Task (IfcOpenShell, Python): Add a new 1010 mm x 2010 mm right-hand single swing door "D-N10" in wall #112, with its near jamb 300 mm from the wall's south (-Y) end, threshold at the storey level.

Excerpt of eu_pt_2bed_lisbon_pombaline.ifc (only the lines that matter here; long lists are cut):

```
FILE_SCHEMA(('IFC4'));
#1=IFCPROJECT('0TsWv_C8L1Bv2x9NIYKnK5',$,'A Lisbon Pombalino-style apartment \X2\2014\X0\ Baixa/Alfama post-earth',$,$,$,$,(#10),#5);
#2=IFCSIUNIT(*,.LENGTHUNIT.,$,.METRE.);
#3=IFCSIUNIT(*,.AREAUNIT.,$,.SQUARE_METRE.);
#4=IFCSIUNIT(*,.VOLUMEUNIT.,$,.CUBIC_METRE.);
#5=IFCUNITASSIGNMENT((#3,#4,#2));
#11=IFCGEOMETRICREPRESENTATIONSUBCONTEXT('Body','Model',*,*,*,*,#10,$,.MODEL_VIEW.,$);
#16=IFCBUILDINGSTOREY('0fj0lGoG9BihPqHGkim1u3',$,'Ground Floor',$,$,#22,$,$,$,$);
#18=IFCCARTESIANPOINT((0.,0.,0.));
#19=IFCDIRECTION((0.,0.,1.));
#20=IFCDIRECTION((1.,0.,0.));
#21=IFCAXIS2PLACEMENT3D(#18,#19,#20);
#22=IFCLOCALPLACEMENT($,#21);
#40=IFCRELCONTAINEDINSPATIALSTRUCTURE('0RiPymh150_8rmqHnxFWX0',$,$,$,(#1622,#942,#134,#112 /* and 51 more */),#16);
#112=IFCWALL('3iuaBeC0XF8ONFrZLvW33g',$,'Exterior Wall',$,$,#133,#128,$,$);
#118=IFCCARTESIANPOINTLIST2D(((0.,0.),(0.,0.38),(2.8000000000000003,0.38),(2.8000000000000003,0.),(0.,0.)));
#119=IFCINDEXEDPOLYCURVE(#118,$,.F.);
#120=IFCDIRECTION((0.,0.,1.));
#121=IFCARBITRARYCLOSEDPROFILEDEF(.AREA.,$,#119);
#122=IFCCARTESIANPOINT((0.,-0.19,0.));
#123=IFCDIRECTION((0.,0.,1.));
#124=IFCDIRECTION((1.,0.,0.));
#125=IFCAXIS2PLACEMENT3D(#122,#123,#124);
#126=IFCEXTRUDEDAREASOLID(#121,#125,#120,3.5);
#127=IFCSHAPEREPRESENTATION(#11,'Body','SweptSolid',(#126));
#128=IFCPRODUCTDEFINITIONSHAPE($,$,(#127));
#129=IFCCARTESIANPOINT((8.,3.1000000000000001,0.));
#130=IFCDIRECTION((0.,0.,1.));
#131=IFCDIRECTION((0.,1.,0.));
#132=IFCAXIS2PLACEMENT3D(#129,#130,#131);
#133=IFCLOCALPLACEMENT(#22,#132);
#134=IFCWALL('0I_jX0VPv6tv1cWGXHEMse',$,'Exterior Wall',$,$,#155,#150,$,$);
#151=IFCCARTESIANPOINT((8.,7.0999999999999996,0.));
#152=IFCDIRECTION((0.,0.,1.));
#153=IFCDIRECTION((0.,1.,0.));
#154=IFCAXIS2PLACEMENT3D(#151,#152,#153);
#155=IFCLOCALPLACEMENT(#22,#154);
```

```python
import numpy as np
import ifcopenshell
import ifcopenshell.api.feature
import ifcopenshell.api.geometry
import ifcopenshell.api.root
import ifcopenshell.api.spatial
import ifcopenshell.geom
import ifcopenshell.util.element
import ifcopenshell.util.placement
import ifcopenshell.util.representation
import ifcopenshell.util.shape
import ifcopenshell.util.unit

model = ifcopenshell.open("eu_pt_2bed_lisbon_pombaline.ifc")
unit_scale = ifcopenshell.util.unit.calculate_unit_scale(model)
settings = ifcopenshell.geom.settings()


def volume(element):
    """Net volume in cubic metres, openings subtracted."""
    shape = ifcopenshell.geom.create_shape(settings, element)
    return ifcopenshell.util.shape.get_volume(shape.geometry)


wall = model.by_guid("3iuaBeC0XF8ONFrZLvW33g")
storey = ifcopenshell.util.element.get_container(wall, ifc_class="IfcBuildingStorey")
context = ifcopenshell.util.representation.get_context(model, "Model", "Body", "MODEL_VIEW")
before = volume(wall)

width, height, from_end, sill = 1.01, 2.01, 0.3, 0.0  # metres

# The wall runs along its own X axis, and the end named is its -X end.
wall_shape = ifcopenshell.geom.create_shape(settings, wall)
x, y, z = ifcopenshell.util.shape.get_vertices(wall_shape.geometry).T
start = x.min() + from_end
face, thickness = float(y.min()), float(y.max() - y.min())
wall_matrix = ifcopenshell.util.placement.get_local_placement(wall.ObjectPlacement)
level = ifcopenshell.util.placement.get_local_placement(storey.ObjectPlacement)[2, 3]


def in_wall(x, y):
    """Placement at x, y metres in the wall's axes, at sill height."""
    matrix = wall_matrix.copy()
    matrix[:, 3] = wall_matrix @ np.array([x / unit_scale, y / unit_scale, 0.0, 1.0])
    matrix[2, 3] = level + sill / unit_scale
    return matrix


# Opening: a box that overshoots both wall faces by 50 mm.
opening = ifcopenshell.api.root.create_entity(model, ifc_class="IfcOpeningElement", predefined_type="OPENING")
box = ifcopenshell.api.geometry.add_wall_representation(
    model, context=context, length=width, height=height, thickness=thickness + 0.1
)
ifcopenshell.api.geometry.assign_representation(model, product=opening, representation=box)
ifcopenshell.api.geometry.edit_object_placement(model, product=opening, matrix=in_wall(start, face - 0.05), is_si=False)
ifcopenshell.api.feature.add_feature(model, feature=opening, element=wall)

door = ifcopenshell.api.root.create_entity(model, ifc_class="IfcDoor", name="D-N10", predefined_type="DOOR")
door.OverallWidth, door.OverallHeight = width / unit_scale, height / unit_scale
door.OperationType = "SINGLE_SWING_RIGHT"
body = ifcopenshell.api.geometry.add_door_representation(
    model,
    context=context,
    overall_width=door.OverallWidth,
    overall_height=door.OverallHeight,
    operation_type="SINGLE_SWING_RIGHT",
    lining_properties={"LiningDepth": thickness / unit_scale, "ThresholdDepth": thickness / unit_scale},
)
ifcopenshell.api.geometry.assign_representation(model, product=door, representation=body)
ifcopenshell.api.spatial.assign_container(model, products=[door], relating_structure=storey)
ifcopenshell.api.feature.add_filling(model, opening=opening, element=door)

# The lining spans the wall, so the door starts at the wall face.
ifcopenshell.api.geometry.edit_object_placement(model, product=door, matrix=in_wall(start, face), is_si=False)

after = volume(wall)

print(f"wall volume {before:.3f} -> {after:.3f} m3")

model.write("eu_pt_2bed_lisbon_pombaline_edited.ifc")
```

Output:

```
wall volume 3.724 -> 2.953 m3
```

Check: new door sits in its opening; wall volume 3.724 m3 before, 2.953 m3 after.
